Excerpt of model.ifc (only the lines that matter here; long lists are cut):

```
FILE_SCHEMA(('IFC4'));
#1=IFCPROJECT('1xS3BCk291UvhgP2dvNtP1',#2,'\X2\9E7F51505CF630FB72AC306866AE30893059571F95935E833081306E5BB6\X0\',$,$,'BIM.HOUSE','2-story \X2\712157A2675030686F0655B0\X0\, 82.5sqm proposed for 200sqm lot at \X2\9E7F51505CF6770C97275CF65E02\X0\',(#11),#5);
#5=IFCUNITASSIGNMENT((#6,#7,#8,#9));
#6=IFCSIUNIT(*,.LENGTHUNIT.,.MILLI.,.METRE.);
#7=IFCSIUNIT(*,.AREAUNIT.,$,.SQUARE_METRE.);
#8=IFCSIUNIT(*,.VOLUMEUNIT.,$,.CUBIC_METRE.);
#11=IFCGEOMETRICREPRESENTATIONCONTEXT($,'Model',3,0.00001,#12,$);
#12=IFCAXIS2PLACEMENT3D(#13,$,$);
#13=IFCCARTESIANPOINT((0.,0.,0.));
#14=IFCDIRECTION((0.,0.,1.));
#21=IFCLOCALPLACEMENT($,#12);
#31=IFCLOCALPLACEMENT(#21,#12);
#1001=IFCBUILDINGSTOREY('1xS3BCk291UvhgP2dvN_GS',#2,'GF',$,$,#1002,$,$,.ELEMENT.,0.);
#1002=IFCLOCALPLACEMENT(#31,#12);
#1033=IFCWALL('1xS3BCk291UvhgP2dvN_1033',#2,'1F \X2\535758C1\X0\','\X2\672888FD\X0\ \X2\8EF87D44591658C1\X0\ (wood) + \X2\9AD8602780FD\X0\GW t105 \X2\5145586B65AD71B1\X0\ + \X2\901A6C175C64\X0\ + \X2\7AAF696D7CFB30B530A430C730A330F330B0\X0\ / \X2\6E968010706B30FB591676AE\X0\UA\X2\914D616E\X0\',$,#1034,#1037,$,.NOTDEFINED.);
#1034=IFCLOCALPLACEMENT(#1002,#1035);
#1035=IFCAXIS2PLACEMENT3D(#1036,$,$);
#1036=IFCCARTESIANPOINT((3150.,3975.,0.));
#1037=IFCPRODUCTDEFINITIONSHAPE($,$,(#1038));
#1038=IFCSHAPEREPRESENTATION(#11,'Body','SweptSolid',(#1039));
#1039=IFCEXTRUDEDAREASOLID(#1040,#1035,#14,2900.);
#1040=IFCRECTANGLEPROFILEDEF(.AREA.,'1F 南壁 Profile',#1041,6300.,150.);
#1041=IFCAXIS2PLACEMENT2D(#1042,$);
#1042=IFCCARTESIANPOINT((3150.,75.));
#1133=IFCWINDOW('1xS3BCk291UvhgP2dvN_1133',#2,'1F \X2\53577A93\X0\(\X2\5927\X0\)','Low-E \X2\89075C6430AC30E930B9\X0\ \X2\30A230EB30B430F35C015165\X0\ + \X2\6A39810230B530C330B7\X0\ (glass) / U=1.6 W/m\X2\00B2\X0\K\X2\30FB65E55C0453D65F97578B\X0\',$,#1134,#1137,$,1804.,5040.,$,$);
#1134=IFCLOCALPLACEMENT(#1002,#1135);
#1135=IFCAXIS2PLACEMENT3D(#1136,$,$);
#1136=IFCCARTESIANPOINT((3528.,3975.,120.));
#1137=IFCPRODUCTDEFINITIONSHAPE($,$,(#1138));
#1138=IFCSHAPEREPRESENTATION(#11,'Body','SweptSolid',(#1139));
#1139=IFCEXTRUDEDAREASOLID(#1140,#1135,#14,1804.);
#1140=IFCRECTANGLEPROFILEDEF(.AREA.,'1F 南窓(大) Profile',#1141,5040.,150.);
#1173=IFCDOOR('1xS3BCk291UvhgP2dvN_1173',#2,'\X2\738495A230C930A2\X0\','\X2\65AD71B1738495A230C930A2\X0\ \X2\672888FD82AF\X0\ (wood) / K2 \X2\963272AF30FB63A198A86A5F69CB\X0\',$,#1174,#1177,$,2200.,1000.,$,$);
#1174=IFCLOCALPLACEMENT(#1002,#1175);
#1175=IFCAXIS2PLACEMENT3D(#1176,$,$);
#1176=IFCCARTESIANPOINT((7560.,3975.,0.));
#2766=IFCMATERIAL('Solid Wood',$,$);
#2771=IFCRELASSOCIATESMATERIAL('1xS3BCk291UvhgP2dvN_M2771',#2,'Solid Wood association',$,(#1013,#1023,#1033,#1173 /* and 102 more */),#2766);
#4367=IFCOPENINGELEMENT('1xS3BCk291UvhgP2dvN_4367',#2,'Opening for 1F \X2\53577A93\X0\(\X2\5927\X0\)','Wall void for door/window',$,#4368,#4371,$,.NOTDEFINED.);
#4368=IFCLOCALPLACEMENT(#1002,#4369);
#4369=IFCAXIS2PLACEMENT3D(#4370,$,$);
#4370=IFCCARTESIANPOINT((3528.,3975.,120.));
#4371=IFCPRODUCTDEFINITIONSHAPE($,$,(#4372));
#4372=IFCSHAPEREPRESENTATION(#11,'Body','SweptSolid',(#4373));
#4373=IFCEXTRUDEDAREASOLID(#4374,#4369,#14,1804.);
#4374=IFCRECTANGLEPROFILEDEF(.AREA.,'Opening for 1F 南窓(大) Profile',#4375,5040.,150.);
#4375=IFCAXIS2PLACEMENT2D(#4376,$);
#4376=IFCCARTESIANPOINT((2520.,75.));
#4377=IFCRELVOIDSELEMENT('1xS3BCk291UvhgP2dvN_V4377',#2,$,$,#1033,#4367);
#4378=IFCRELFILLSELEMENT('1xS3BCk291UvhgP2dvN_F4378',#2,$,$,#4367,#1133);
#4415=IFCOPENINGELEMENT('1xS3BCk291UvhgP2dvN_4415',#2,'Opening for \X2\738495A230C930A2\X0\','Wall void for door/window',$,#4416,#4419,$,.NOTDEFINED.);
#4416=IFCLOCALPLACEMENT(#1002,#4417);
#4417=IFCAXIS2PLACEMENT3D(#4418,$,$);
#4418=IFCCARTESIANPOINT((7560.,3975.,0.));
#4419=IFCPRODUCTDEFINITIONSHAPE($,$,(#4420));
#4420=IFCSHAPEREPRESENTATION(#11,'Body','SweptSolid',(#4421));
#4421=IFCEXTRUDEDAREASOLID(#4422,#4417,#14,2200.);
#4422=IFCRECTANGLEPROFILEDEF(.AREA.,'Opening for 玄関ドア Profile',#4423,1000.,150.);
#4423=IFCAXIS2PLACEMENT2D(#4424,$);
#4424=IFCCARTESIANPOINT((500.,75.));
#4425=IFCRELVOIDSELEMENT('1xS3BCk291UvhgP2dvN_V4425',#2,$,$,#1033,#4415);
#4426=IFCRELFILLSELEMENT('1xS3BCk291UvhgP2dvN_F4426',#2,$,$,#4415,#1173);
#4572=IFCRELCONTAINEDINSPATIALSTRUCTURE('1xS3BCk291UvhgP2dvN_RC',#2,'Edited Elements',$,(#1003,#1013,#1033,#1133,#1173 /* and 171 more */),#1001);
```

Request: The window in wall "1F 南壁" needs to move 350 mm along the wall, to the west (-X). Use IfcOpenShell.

```python
import ifcopenshell
import ifcopenshell.api.geometry
import ifcopenshell.util.placement

model = ifcopenshell.open("model.ifc")

window = model.by_guid("1xS3BCk291UvhgP2dvN_1133")
opening = window.FillsVoids[0].RelatingOpeningElement
wall = opening.VoidsElements[0].RelatingBuildingElement

wall_matrix = ifcopenshell.util.placement.get_local_placement(wall.ObjectPlacement)
shift = wall_matrix[:3, 0] * -350.0
before = ifcopenshell.util.placement.get_local_placement(window.ObjectPlacement)[:3, 3].copy()

# The window is not placed relative to its opening, so move both.
for product in (opening, window):
    matrix = ifcopenshell.util.placement.get_local_placement(product.ObjectPlacement)
    matrix[:3, 3] += shift
    ifcopenshell.api.geometry.edit_object_placement(model, product=product, matrix=matrix, is_si=False)

after = ifcopenshell.util.placement.get_local_placement(window.ObjectPlacement)[:3, 3]
print("window moved by", (after - before).round(3) + 0.0)

model.write("model_edited.ifc")
```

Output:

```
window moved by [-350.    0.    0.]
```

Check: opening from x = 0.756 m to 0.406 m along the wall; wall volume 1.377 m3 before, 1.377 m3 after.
